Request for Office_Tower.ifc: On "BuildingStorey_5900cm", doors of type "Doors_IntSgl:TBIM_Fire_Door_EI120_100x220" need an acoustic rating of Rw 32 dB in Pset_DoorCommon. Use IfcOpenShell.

First a look at what the model holds.

```python
import ifcopenshell
import ifcopenshell.util.element

model = ifcopenshell.open("Office_Tower.ifc")
print(model.schema)
storey = next(s for s in model.by_type("IfcBuildingStorey") if s.Name == "BuildingStorey_5900cm")
doors = [e for e in ifcopenshell.util.element.get_decomposition(storey) if e.is_a("IfcDoor")]
seen = {}
for e in doors:
    element_type = ifcopenshell.util.element.get_type(e)
    key = (element_type.Name if element_type != e and element_type else None, ifcopenshell.util.element.get_pset(e, "Pset_DoorCommon", "AcousticRating"))
    seen[key] = seen.get(key, 0) + 1
for (name, value), count in sorted(seen.items(), key=str):
    print(count, "x", name, "|", value)
```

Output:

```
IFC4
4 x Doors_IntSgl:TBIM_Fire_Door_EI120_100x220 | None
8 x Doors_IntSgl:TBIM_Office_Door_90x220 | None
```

```python
import ifcopenshell
import ifcopenshell.api.pset
import ifcopenshell.util.element

model = ifcopenshell.open("Office_Tower.ifc")

storey = next(s for s in model.by_type("IfcBuildingStorey") if s.Name == "BuildingStorey_5900cm")
doors = [e for e in ifcopenshell.util.element.get_decomposition(storey) if e.is_a("IfcDoor")]

count = 0
for e in doors:
    element_type = ifcopenshell.util.element.get_type(e)
    if element_type in (None, e) or element_type.Name != "Doors_IntSgl:TBIM_Fire_Door_EI120_100x220":
        continue
    # add_pset returns the element's existing set when there is one.
    pset = ifcopenshell.api.pset.add_pset(model, product=e, name="Pset_DoorCommon")
    ifcopenshell.api.pset.edit_pset(model, pset=pset, properties={"AcousticRating": "Rw 32 dB"})
    count += 1

print(count, "doors updated")

model.write("Office_Tower_v2.ifc")
```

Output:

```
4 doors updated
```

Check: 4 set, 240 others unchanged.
